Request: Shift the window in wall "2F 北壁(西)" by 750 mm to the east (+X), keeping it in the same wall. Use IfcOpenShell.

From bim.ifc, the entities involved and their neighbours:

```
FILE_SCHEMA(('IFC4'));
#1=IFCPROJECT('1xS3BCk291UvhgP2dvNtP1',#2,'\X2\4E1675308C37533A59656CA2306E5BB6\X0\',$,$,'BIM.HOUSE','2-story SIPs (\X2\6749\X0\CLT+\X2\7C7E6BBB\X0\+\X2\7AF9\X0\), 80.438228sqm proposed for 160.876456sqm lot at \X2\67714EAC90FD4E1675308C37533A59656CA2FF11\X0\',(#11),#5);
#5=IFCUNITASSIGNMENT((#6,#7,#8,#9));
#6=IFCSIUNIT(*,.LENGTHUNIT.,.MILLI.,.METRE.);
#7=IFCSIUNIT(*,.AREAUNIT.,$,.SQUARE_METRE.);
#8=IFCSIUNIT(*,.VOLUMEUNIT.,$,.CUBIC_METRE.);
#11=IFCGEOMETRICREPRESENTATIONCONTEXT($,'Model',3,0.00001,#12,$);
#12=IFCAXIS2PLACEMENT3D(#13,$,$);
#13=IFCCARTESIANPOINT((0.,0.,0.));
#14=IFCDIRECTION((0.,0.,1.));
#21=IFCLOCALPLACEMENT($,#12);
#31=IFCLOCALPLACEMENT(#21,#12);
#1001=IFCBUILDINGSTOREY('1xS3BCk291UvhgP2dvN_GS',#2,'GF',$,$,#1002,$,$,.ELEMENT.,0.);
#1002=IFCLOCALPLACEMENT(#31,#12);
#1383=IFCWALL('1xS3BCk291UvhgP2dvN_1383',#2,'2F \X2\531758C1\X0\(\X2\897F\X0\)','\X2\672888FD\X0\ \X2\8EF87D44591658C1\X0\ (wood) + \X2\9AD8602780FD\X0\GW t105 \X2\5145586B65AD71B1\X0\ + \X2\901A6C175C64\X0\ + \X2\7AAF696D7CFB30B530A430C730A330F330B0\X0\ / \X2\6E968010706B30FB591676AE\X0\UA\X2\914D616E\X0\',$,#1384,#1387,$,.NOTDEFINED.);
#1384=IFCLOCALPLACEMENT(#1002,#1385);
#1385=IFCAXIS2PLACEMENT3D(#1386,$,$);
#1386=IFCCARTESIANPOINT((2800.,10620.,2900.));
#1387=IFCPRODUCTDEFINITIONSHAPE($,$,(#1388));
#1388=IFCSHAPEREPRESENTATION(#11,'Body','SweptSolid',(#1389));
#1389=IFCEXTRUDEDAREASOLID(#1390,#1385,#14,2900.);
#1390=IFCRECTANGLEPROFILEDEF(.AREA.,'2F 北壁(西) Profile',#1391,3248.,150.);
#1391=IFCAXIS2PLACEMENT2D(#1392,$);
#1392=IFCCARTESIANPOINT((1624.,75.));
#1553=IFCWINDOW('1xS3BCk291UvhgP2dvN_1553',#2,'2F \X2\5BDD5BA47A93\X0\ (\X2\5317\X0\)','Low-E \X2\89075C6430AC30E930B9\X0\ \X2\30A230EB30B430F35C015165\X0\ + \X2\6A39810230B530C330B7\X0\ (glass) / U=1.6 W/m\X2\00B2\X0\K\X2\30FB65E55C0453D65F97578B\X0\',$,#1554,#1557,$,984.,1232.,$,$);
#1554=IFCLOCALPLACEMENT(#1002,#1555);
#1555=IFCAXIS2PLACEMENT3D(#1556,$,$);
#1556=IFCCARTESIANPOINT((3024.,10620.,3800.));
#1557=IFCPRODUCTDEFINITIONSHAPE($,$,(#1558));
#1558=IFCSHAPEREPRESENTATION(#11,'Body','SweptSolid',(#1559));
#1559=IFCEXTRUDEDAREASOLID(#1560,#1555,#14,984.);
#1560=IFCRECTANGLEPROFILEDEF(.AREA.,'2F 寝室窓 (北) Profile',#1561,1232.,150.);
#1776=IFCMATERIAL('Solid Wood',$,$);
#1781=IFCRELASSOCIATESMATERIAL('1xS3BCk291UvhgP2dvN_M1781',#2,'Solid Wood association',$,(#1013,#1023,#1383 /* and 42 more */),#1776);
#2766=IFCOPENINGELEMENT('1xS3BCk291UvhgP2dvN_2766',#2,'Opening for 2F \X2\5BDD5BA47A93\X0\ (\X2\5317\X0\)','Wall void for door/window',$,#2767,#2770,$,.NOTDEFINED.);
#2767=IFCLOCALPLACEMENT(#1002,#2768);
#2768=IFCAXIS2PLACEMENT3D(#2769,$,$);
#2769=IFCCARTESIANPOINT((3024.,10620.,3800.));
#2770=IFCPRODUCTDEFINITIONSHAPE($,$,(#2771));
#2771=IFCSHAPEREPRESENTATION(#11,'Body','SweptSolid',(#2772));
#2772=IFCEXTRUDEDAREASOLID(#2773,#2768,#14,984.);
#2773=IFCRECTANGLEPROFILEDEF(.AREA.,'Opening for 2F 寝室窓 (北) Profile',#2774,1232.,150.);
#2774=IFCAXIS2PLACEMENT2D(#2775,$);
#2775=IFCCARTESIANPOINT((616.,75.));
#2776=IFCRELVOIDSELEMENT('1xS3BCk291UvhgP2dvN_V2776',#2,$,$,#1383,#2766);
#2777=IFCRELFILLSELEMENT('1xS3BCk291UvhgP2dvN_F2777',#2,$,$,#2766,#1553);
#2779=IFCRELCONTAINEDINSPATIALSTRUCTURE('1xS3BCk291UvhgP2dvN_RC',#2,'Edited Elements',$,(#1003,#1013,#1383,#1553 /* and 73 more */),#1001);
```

```python
import ifcopenshell
import ifcopenshell.api.geometry
import ifcopenshell.util.placement
import ifcopenshell.util.unit

model = ifcopenshell.open("bim.ifc")
unit_scale = ifcopenshell.util.unit.calculate_unit_scale(model)

window = model.by_guid("1xS3BCk291UvhgP2dvN_1553")
opening = window.FillsVoids[0].RelatingOpeningElement
wall = opening.VoidsElements[0].RelatingBuildingElement

wall_matrix = ifcopenshell.util.placement.get_local_placement(wall.ObjectPlacement)
shift = wall_matrix[:3, 0] * 0.75 / unit_scale
before = ifcopenshell.util.placement.get_local_placement(window.ObjectPlacement)[:3, 3].copy()

# The window is not placed relative to its opening, so move both.
for product in (opening, window):
    matrix = ifcopenshell.util.placement.get_local_placement(product.ObjectPlacement)
    matrix[:3, 3] += shift
    ifcopenshell.api.geometry.edit_object_placement(model, product=product, matrix=matrix, is_si=False)

after = ifcopenshell.util.placement.get_local_placement(window.ObjectPlacement)[:3, 3]
print("window moved by", (after - before).round(3) + 0.0)

model.write("bim-out.ifc")
```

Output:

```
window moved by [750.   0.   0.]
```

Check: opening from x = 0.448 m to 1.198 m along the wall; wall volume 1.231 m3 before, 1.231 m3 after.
